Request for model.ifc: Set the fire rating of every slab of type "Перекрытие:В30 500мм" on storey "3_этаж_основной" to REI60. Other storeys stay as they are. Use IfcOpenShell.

First a look at what the model holds.

```python
import ifcopenshell
import ifcopenshell.util.element

model = ifcopenshell.open("model.ifc")
print(model.schema)
storey = next(s for s in model.by_type("IfcBuildingStorey") if s.Name == "3_этаж_основной")
slabs = [e for e in ifcopenshell.util.element.get_decomposition(storey) if e.is_a("IfcSlab")]
seen = {}
for e in slabs:
    element_type = ifcopenshell.util.element.get_type(e)
    key = (element_type.Name if element_type != e and element_type else None, ifcopenshell.util.element.get_pset(e, "Pset_SlabCommon", "FireRating"))
    seen[key] = seen.get(key, 0) + 1
for (name, value), count in sorted(seen.items(), key=str):
    print(count, "x", name, "|", value)
```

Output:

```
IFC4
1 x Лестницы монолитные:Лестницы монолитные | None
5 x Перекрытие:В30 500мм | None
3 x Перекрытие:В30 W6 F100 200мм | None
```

```python
import ifcopenshell
import ifcopenshell.api.pset
import ifcopenshell.util.element

model = ifcopenshell.open("model.ifc")

storey = next(s for s in model.by_type("IfcBuildingStorey") if s.Name == "3_этаж_основной")
slabs = [e for e in ifcopenshell.util.element.get_decomposition(storey) if e.is_a("IfcSlab")]

count = 0
for e in slabs:
    element_type = ifcopenshell.util.element.get_type(e)
    if element_type in (None, e) or element_type.Name != "Перекрытие:В30 500мм":
        continue
    # add_pset returns the element's existing set when there is one.
    pset = ifcopenshell.api.pset.add_pset(model, product=e, name="Pset_SlabCommon")
    ifcopenshell.api.pset.edit_pset(model, pset=pset, properties={"FireRating": "REI60"})
    count += 1

print(count, "slabs updated")

model.write("model_v2.ifc")
```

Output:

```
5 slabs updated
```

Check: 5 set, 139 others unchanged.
